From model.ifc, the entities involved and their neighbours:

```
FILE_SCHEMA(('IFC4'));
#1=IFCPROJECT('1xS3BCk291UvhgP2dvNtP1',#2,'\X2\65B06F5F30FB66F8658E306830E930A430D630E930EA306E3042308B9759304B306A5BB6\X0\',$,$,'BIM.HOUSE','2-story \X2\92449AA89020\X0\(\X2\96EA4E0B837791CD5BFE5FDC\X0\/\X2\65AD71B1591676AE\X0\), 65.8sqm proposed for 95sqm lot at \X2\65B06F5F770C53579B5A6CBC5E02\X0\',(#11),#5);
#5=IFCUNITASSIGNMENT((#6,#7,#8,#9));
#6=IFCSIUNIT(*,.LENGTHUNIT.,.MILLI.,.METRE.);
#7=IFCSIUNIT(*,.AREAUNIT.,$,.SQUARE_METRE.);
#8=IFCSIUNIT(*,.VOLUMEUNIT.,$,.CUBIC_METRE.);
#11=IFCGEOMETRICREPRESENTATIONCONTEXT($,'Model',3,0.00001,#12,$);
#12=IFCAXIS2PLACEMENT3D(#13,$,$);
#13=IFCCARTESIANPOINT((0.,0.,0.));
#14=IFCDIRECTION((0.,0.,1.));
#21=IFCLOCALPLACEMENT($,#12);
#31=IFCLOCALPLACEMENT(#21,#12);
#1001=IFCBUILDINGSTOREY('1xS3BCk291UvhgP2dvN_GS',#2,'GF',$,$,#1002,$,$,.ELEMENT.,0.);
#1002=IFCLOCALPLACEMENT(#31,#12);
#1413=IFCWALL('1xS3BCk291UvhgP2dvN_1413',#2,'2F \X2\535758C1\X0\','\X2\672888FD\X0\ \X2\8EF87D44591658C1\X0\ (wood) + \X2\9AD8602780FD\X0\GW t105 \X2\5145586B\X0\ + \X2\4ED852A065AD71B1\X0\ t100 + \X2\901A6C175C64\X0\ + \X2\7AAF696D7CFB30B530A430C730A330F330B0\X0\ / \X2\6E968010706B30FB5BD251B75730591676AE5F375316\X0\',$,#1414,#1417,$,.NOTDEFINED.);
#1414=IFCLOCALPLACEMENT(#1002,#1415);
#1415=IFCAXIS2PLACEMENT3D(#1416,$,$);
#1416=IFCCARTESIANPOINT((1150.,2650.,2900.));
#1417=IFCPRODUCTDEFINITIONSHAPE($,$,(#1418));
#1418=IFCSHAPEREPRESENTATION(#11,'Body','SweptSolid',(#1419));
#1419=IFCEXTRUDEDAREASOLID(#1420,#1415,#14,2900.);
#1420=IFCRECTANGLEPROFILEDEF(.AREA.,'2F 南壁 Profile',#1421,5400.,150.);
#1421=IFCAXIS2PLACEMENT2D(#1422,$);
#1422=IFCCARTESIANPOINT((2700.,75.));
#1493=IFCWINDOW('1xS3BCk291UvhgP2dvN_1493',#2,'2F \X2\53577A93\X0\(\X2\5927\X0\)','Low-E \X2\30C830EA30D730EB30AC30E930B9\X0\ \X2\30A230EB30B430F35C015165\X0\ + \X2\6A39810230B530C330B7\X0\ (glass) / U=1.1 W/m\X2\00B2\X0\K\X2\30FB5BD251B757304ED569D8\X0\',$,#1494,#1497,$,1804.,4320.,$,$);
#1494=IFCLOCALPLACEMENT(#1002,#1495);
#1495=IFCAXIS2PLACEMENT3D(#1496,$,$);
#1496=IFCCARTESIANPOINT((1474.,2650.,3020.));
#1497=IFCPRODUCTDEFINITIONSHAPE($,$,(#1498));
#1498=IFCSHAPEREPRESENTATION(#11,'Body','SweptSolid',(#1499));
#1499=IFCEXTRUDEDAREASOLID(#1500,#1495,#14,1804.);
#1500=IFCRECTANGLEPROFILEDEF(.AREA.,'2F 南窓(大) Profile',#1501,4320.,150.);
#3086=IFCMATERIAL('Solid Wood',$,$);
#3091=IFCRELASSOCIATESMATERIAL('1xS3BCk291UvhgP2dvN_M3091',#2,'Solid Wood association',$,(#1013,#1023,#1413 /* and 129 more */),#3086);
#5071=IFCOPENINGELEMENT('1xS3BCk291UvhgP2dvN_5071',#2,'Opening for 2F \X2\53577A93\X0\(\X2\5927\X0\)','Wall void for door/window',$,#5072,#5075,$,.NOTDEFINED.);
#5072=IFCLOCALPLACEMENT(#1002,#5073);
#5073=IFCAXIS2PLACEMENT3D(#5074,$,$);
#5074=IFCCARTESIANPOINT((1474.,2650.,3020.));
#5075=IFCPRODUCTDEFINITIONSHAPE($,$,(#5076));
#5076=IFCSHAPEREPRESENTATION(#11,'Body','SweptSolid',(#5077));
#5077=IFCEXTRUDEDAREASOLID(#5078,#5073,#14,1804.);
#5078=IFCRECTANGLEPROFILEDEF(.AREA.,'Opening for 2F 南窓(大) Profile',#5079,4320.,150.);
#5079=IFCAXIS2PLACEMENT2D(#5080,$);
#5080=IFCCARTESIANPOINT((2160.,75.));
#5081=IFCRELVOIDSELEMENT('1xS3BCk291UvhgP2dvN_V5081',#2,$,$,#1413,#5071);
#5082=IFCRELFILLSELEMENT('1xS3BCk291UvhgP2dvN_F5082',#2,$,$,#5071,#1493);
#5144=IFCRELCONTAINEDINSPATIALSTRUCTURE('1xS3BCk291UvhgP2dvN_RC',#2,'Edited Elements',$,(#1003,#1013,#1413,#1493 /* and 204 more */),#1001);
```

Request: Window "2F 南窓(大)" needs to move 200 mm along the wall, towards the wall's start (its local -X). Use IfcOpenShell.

```python
import ifcopenshell
import ifcopenshell.api.geometry
import ifcopenshell.util.placement

model = ifcopenshell.open("model.ifc")

window = model.by_guid("1xS3BCk291UvhgP2dvN_1493")
opening = window.FillsVoids[0].RelatingOpeningElement
wall = opening.VoidsElements[0].RelatingBuildingElement

wall_matrix = ifcopenshell.util.placement.get_local_placement(wall.ObjectPlacement)
shift = wall_matrix[:3, 0] * -200.0
before = ifcopenshell.util.placement.get_local_placement(window.ObjectPlacement)[:3, 3].copy()

# The window is not placed relative to its opening, so move both.
for product in (opening, window):
    matrix = ifcopenshell.util.placement.get_local_placement(product.ObjectPlacement)
    matrix[:3, 3] += shift
    ifcopenshell.api.geometry.edit_object_placement(model, product=product, matrix=matrix, is_si=False)

after = ifcopenshell.util.placement.get_local_placement(window.ObjectPlacement)[:3, 3]
print("window moved by", (after - before).round(3) + 0.0)

model.write("model_v2.ifc")
```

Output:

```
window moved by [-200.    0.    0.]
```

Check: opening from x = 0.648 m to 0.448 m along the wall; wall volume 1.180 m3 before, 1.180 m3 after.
